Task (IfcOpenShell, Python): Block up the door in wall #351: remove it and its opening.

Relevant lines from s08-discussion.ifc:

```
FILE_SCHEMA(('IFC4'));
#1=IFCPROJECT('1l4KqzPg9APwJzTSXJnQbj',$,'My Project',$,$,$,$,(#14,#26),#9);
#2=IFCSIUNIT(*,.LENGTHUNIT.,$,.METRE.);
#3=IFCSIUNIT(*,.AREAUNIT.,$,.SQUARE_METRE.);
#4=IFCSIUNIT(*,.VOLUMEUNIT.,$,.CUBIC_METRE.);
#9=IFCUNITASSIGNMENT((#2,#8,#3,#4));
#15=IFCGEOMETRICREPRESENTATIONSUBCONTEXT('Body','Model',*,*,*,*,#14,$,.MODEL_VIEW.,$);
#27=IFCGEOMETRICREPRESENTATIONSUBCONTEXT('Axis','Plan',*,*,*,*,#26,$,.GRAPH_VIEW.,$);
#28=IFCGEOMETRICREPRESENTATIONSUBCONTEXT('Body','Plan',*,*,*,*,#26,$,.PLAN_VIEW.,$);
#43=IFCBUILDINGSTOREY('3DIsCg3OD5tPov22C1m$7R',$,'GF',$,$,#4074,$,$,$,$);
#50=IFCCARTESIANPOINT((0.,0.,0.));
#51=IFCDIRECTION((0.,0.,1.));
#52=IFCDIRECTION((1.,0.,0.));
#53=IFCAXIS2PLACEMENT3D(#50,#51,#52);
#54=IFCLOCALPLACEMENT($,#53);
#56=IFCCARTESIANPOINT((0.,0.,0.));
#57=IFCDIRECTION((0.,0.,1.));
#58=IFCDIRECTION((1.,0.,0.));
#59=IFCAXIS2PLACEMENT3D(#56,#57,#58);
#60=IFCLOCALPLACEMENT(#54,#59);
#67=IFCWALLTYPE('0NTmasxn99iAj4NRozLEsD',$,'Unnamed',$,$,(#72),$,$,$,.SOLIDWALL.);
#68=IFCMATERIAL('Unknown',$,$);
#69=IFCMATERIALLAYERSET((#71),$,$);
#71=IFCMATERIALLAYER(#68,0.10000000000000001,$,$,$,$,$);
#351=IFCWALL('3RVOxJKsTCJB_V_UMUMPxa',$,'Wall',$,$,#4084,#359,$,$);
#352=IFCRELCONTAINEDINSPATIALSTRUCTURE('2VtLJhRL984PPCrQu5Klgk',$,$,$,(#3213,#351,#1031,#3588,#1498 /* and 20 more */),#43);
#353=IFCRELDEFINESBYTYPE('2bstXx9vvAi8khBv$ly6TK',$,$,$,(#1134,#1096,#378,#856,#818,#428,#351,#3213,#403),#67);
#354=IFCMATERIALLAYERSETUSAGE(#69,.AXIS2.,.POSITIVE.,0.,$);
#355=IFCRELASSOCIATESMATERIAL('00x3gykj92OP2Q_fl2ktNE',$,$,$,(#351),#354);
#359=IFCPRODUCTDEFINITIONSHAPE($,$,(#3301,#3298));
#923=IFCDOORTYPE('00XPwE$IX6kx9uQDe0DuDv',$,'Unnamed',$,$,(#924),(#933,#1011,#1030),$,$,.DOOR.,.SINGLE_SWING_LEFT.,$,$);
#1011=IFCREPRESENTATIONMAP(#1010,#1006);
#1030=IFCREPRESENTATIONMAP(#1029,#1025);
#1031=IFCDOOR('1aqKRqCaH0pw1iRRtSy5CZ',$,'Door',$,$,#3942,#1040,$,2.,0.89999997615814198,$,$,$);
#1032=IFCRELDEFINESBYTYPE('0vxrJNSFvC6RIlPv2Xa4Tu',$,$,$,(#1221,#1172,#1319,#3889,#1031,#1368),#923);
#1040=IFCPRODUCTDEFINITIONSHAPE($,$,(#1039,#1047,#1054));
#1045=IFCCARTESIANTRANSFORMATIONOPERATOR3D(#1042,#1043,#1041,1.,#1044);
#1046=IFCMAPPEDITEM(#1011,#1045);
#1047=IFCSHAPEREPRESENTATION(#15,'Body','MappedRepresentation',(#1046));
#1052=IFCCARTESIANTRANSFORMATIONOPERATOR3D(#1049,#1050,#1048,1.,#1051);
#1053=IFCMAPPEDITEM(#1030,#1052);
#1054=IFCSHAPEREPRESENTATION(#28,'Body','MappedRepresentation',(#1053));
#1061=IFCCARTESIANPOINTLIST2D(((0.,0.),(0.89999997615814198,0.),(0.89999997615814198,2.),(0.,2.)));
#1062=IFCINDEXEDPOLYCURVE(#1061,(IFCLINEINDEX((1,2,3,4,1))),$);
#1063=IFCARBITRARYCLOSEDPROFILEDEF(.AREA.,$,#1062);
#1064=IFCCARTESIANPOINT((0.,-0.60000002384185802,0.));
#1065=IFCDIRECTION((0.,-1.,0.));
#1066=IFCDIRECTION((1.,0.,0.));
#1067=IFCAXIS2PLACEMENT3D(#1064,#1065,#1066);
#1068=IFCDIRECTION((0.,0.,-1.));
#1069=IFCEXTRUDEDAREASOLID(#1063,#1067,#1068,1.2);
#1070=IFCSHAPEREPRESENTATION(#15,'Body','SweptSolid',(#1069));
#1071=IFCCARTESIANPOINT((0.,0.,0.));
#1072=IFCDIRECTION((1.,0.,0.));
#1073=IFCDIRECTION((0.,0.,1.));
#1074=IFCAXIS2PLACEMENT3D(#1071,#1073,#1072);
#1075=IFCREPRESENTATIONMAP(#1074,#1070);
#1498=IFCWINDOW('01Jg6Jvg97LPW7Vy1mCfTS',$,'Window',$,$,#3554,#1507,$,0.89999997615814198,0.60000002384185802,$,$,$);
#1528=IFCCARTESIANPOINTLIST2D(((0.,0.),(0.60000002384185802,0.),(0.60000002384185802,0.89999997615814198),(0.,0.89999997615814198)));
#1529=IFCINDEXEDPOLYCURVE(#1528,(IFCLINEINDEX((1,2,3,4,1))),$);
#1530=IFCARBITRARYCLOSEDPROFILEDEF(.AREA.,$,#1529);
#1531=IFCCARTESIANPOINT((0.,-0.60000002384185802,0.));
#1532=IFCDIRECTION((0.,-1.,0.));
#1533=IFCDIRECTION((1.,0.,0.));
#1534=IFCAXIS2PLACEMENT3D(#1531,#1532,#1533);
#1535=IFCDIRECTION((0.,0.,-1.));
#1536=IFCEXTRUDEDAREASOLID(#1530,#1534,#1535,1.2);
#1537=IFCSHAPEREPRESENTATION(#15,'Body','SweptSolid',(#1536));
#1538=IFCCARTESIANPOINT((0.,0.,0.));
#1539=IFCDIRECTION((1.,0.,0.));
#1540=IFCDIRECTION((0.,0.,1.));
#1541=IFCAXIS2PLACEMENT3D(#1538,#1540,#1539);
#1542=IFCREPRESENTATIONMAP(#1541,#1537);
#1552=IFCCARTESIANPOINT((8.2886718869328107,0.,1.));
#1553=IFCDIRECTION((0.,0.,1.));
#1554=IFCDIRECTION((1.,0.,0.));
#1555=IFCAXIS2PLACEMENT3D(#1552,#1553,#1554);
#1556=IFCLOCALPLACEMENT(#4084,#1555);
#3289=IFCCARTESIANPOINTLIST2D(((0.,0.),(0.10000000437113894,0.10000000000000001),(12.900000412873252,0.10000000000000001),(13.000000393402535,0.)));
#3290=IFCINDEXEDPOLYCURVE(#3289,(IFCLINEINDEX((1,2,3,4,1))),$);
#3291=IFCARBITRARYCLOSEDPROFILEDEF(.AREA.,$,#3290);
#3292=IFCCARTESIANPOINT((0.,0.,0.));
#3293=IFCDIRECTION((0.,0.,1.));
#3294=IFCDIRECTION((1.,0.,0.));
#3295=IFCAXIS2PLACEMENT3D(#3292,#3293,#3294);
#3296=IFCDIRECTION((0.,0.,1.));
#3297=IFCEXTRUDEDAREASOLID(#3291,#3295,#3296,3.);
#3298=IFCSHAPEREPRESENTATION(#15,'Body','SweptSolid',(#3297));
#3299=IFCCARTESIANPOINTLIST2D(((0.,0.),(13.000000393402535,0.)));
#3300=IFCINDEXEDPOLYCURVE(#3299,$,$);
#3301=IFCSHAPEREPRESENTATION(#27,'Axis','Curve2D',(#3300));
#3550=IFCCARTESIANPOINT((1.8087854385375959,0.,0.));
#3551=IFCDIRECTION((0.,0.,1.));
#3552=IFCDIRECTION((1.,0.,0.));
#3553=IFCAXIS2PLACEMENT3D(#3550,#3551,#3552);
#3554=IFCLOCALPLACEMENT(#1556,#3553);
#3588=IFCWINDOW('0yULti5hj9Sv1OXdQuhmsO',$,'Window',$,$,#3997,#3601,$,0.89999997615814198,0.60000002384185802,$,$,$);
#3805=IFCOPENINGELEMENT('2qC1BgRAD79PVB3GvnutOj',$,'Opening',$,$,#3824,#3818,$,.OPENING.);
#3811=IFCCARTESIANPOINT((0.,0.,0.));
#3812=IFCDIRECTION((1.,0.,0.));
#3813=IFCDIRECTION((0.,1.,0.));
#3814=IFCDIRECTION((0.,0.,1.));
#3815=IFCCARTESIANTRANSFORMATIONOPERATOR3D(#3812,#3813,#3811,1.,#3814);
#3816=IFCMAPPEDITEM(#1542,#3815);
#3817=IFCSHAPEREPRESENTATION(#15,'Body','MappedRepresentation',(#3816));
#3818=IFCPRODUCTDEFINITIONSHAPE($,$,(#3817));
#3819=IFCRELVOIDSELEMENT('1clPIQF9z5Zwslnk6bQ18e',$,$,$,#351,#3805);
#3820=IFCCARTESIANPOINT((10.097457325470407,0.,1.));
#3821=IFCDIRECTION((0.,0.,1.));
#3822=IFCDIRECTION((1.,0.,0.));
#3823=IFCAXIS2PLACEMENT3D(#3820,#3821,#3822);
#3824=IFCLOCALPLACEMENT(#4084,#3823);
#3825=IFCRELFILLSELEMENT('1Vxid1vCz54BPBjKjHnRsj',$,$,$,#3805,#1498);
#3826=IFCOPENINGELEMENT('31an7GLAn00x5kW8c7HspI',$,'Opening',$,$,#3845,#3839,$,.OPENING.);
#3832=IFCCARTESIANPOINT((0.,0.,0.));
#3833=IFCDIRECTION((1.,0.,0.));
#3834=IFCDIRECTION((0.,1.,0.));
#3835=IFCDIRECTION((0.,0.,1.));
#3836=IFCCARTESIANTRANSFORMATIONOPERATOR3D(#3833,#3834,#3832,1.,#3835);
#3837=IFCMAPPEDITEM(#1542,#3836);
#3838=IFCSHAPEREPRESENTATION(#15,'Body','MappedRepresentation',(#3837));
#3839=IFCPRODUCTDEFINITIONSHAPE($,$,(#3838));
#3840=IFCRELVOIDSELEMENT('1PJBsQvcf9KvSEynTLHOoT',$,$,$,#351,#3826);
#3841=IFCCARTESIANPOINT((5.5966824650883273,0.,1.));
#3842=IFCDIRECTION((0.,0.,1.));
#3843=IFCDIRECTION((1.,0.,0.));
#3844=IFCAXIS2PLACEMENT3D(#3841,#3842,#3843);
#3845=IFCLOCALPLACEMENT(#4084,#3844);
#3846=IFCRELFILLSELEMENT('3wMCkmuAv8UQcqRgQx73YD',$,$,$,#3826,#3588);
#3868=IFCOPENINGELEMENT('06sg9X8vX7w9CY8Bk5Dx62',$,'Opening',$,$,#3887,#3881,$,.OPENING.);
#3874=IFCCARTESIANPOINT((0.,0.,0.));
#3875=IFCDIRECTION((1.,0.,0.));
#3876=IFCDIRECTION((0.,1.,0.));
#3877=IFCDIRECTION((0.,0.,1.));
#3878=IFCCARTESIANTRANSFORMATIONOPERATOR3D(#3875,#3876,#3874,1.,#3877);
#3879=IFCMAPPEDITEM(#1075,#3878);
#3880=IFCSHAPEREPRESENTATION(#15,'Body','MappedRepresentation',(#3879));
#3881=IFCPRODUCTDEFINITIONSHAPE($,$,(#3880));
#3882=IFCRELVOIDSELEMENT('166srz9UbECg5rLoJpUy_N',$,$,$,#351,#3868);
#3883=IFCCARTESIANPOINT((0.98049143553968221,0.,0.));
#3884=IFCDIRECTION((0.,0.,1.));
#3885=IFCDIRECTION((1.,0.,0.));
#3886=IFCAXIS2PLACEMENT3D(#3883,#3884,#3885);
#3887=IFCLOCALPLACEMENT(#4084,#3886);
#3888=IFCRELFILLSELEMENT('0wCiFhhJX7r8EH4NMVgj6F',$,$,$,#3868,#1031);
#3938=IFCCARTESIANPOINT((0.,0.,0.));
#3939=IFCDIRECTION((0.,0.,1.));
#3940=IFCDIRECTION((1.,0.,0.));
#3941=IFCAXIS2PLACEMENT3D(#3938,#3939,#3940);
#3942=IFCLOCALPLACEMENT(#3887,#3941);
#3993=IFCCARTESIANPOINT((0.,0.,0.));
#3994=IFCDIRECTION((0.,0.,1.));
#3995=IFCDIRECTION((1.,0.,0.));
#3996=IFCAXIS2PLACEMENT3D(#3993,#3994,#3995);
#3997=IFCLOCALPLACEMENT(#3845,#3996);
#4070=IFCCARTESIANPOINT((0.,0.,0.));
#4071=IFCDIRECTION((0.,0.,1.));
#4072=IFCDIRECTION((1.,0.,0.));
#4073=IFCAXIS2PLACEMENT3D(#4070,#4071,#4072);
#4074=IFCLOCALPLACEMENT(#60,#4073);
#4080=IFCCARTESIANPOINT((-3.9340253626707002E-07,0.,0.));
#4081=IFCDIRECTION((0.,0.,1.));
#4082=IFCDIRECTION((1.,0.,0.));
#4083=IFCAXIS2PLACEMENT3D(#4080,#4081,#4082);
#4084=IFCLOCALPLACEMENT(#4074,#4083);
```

```python
import ifcopenshell
import ifcopenshell.api.feature
import ifcopenshell.api.root
import ifcopenshell.geom
import ifcopenshell.util.shape

model = ifcopenshell.open("s08-discussion.ifc")
settings = ifcopenshell.geom.settings()


def volume(element):
    """Net volume in cubic metres, openings subtracted."""
    shape = ifcopenshell.geom.create_shape(settings, element)
    return ifcopenshell.util.shape.get_volume(shape.geometry)


door = model.by_id(1031)
opening = door.FillsVoids[0].RelatingOpeningElement
wall = opening.VoidsElements[0].RelatingBuildingElement
before = volume(wall)

ifcopenshell.api.root.remove_product(model, product=door)
ifcopenshell.api.feature.remove_feature(model, feature=opening)

after = volume(wall)

print(f"wall volume {before:.3f} -> {after:.3f} m3")

model.write("s08-discussion_rev.ifc")
```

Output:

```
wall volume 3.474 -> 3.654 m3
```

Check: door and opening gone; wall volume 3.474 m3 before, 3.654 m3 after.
